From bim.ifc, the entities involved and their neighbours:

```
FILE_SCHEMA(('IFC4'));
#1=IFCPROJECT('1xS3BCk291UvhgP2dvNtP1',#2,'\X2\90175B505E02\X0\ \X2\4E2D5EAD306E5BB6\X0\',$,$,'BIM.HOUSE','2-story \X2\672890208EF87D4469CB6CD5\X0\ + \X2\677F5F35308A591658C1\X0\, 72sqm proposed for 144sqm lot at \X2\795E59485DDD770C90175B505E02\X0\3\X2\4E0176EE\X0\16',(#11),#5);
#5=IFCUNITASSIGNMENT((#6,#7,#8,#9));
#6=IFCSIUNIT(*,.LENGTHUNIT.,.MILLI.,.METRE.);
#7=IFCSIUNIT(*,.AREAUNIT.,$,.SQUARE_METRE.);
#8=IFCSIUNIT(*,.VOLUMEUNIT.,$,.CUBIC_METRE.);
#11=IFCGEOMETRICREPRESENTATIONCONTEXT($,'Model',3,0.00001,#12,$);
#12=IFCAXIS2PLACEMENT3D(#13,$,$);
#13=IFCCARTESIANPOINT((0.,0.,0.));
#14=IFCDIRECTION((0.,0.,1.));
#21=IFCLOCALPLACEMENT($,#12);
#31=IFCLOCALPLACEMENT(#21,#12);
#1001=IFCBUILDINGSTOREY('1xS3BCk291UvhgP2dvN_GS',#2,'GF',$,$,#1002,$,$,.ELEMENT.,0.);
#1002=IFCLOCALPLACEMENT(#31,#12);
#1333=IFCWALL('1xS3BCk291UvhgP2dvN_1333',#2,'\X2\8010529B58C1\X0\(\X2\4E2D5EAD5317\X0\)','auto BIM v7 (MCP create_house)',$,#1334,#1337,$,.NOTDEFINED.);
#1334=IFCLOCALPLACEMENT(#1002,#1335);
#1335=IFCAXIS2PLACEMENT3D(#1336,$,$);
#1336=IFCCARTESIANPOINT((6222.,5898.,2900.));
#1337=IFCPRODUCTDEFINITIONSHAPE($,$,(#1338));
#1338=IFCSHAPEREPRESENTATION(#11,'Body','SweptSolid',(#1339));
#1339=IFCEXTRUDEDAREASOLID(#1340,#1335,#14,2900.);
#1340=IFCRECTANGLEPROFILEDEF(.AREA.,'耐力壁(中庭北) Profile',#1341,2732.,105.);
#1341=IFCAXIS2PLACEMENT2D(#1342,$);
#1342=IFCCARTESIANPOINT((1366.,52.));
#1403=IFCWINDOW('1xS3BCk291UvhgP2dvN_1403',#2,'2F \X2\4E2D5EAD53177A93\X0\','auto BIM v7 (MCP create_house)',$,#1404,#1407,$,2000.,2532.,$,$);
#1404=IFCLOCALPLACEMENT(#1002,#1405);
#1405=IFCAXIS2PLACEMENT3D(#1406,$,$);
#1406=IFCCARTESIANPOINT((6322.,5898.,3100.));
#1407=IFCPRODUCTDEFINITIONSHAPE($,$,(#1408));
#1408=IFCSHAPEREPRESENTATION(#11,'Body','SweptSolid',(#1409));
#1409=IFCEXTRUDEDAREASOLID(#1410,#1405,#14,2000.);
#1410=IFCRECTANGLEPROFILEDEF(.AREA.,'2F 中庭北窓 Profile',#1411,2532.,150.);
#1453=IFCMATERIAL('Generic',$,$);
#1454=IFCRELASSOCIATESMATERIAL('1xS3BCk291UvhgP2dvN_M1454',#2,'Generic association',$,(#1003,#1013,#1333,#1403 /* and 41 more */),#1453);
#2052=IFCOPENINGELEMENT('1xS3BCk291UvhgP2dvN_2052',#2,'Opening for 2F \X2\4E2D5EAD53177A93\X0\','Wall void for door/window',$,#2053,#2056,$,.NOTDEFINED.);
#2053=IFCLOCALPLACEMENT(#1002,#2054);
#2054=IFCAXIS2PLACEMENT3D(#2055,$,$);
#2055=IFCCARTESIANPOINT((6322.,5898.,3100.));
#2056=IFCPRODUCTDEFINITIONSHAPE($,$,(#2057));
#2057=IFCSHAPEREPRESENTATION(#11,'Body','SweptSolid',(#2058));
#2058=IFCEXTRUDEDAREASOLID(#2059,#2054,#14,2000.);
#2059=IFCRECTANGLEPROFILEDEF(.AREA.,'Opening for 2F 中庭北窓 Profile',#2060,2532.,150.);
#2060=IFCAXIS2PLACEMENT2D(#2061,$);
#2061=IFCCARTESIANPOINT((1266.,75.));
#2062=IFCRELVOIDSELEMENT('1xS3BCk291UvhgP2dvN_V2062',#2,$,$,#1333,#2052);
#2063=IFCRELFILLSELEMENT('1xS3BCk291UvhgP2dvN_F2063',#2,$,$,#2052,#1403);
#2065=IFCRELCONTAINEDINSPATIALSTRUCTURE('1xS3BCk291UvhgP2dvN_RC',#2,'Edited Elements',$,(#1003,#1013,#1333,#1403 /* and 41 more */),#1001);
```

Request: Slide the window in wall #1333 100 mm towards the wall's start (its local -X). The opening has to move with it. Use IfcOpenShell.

```python
import ifcopenshell
import ifcopenshell.api.geometry
import ifcopenshell.util.placement
import ifcopenshell.util.unit

model = ifcopenshell.open("bim.ifc")
unit_scale = ifcopenshell.util.unit.calculate_unit_scale(model)

window = model.by_guid("1xS3BCk291UvhgP2dvN_1403")
opening = window.FillsVoids[0].RelatingOpeningElement
wall = opening.VoidsElements[0].RelatingBuildingElement

wall_matrix = ifcopenshell.util.placement.get_local_placement(wall.ObjectPlacement)
shift = wall_matrix[:3, 0] * -0.1 / unit_scale
before = ifcopenshell.util.placement.get_local_placement(window.ObjectPlacement)[:3, 3].copy()

# The window is not placed relative to its opening, so move both.
for product in (opening, window):
    matrix = ifcopenshell.util.placement.get_local_placement(product.ObjectPlacement)
    matrix[:3, 3] += shift
    ifcopenshell.api.geometry.edit_object_placement(model, product=product, matrix=matrix, is_si=False)

after = ifcopenshell.util.placement.get_local_placement(window.ObjectPlacement)[:3, 3]
print("window moved by", (after - before).round(3) + 0.0)

model.write("bim-out.ifc")
```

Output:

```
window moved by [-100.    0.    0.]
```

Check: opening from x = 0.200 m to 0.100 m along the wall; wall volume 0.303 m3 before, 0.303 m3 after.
